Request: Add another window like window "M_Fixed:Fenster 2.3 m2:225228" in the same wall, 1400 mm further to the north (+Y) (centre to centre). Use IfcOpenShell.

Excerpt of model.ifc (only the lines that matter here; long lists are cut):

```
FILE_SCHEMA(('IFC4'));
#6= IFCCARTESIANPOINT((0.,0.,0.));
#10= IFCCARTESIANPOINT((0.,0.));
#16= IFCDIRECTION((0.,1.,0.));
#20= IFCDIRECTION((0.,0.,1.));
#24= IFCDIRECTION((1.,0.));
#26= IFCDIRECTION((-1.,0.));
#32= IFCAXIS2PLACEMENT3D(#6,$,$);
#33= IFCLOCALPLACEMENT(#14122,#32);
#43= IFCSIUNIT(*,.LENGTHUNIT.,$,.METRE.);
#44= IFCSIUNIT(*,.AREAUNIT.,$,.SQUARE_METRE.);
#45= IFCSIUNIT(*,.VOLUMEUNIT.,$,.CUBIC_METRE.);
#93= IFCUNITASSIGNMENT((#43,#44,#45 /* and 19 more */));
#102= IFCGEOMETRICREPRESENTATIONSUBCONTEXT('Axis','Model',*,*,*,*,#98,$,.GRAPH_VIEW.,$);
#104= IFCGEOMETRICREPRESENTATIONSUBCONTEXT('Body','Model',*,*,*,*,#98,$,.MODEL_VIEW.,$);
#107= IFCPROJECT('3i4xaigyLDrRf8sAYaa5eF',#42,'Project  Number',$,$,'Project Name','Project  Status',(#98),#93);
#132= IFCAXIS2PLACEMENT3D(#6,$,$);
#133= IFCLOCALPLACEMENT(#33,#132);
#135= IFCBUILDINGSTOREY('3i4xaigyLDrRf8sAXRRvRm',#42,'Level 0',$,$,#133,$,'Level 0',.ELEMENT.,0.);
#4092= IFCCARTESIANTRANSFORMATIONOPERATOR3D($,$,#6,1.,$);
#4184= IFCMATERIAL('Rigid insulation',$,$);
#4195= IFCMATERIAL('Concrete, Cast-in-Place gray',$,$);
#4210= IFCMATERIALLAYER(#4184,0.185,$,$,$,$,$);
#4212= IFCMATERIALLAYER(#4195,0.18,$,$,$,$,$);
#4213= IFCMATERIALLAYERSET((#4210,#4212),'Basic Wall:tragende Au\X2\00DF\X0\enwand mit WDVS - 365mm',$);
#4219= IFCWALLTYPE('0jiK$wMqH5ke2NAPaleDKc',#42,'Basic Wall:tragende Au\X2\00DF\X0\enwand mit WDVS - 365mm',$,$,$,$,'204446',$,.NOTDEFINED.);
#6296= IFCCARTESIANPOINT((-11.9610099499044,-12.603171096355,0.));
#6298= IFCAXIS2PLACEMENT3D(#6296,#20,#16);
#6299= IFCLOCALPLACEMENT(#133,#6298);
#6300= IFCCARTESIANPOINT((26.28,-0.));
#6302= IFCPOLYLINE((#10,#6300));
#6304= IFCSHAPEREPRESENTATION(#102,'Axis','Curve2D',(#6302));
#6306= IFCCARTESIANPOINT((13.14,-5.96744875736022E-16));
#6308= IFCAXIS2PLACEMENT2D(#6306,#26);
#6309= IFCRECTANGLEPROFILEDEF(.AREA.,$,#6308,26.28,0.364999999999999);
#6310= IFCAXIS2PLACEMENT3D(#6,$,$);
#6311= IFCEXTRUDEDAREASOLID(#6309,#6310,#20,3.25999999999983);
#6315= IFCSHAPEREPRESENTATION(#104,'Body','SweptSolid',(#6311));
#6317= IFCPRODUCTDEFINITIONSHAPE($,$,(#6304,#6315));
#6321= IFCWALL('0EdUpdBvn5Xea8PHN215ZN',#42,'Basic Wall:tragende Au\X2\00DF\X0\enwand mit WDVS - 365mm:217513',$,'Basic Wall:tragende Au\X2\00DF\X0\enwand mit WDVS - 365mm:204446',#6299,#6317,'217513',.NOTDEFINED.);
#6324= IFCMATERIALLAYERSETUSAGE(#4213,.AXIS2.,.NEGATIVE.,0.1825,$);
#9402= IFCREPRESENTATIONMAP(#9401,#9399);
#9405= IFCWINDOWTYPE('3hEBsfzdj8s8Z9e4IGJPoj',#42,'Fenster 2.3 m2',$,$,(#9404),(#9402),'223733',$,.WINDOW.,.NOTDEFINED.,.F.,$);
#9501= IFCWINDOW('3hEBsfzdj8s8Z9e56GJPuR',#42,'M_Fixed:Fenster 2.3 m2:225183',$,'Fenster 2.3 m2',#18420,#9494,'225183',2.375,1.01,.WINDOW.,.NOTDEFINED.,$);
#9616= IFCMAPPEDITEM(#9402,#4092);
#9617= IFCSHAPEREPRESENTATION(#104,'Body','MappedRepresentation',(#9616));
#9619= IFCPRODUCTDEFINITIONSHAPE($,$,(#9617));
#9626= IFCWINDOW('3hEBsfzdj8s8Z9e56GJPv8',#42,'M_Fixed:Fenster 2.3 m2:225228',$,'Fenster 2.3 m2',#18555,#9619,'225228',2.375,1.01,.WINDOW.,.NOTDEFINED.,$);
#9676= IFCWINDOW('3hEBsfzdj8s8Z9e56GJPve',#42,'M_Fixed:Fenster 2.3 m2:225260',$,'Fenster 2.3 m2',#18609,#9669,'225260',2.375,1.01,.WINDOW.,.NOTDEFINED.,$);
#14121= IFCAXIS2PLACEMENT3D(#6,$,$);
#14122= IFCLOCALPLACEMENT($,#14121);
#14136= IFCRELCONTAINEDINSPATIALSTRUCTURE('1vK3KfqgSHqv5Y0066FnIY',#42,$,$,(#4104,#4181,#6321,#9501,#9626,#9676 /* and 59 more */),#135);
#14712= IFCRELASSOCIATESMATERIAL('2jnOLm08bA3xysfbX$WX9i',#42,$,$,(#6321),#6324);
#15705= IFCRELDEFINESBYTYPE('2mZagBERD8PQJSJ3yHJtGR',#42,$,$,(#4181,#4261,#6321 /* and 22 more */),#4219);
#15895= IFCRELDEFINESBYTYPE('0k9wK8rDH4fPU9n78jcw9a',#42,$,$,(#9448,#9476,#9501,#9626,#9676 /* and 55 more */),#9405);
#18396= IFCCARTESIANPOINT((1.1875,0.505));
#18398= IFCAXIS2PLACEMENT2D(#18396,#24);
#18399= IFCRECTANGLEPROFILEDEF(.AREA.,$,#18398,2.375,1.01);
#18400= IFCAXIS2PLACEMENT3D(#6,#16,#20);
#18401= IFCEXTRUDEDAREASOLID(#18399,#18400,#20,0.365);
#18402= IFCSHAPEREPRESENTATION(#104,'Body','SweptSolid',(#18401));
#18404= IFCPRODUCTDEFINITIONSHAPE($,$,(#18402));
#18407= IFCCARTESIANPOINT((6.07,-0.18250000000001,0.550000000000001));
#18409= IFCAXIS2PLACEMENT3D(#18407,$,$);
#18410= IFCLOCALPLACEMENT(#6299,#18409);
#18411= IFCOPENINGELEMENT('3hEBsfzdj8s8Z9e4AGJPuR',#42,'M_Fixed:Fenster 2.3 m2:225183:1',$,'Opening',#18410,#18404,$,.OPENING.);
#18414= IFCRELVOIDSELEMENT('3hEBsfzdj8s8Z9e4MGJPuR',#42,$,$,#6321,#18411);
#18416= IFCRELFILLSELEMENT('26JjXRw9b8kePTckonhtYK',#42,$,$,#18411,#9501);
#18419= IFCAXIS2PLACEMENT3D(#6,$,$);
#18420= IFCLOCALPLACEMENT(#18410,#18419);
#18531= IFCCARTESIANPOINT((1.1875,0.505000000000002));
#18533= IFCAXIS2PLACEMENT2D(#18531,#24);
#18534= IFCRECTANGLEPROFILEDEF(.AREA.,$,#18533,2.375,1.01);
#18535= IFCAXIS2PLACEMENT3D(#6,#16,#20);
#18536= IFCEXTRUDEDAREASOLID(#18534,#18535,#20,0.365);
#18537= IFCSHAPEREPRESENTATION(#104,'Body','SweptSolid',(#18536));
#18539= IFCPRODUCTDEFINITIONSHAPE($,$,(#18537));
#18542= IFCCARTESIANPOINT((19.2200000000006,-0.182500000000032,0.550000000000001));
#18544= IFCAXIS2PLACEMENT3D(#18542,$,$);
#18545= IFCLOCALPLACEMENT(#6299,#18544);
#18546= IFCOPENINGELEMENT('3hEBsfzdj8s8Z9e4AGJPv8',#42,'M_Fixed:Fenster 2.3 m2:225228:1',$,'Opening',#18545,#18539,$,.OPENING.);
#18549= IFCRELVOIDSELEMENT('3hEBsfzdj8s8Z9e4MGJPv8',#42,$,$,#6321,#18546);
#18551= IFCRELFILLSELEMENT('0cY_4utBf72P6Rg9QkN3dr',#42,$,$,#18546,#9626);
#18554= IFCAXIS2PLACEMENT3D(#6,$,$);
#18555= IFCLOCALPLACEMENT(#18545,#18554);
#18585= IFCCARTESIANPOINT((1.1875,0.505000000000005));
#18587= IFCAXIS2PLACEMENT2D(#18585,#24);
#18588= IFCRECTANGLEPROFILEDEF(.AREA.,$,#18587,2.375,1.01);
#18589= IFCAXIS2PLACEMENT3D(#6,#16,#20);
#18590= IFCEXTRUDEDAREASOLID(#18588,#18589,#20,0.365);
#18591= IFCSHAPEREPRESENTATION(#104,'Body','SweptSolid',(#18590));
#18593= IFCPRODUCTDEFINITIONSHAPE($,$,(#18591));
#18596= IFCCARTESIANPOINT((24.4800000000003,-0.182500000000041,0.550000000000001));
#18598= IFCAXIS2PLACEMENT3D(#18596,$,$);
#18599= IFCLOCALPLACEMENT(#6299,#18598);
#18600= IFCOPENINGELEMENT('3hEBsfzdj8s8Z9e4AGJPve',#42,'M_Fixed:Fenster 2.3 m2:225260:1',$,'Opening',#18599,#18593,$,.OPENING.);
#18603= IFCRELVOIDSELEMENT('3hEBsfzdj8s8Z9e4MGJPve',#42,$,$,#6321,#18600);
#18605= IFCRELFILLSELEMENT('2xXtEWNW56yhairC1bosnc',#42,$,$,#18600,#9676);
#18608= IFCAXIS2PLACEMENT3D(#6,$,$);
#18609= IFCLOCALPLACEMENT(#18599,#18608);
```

```python
import ifcopenshell
import ifcopenshell.api.feature
import ifcopenshell.api.geometry
import ifcopenshell.api.root
import ifcopenshell.geom
import ifcopenshell.util.element
import ifcopenshell.util.placement
import ifcopenshell.util.shape
import ifcopenshell.util.unit

model = ifcopenshell.open("model.ifc")
unit_scale = ifcopenshell.util.unit.calculate_unit_scale(model)
settings = ifcopenshell.geom.settings()


def volume(element):
    """Net volume in cubic metres, openings subtracted."""
    shape = ifcopenshell.geom.create_shape(settings, element)
    return ifcopenshell.util.shape.get_volume(shape.geometry)


def reuse_history(source, copy):
    """copy_class also copies each property set's owner history, people and application; keep the originals."""
    for rel in copy.IsDefinedBy:
        if rel.is_a("IfcRelDefinesByProperties") and (history := rel.RelatingPropertyDefinition.OwnerHistory):
            rel.RelatingPropertyDefinition.OwnerHistory = source.OwnerHistory
            ifcopenshell.util.element.remove_deep2(model, history)


window = model.by_guid("3hEBsfzdj8s8Z9e56GJPv8")
opening = window.FillsVoids[0].RelatingOpeningElement
wall = opening.VoidsElements[0].RelatingBuildingElement
before = volume(wall)
shift = ifcopenshell.util.placement.get_local_placement(wall.ObjectPlacement)[:3, 0] * 1.4 / unit_scale

# copy_class copies the void relationship, type, container and properties, but no geometry.
new_opening = ifcopenshell.api.root.copy_class(model, product=opening)
new_opening.Representation = ifcopenshell.util.element.copy_deep(
    model, opening.Representation, exclude=["IfcGeometricRepresentationContext", "IfcRepresentationMap"]
)
new_opening.Name = "M_Fixed:Fenster 2.3 m2"
new_window = ifcopenshell.api.root.copy_class(model, product=window)
new_window.Representation = ifcopenshell.util.element.copy_deep(
    model, window.Representation, exclude=["IfcGeometricRepresentationContext", "IfcRepresentationMap"]
)
new_window.Name = "M_Fixed:Fenster 2.3 m2"
new_window.Tag = None
reuse_history(window, new_window)
ifcopenshell.api.feature.add_filling(model, opening=new_opening, element=new_window)

for old, new in ((opening, new_opening), (window, new_window)):
    matrix = ifcopenshell.util.placement.get_local_placement(old.ObjectPlacement)
    matrix[:3, 3] += shift
    ifcopenshell.api.geometry.edit_object_placement(model, product=new, matrix=matrix, is_si=False)

after = volume(wall)

print(f"wall volume {before:.3f} -> {after:.3f} m3")

model.write("model_rev.ifc")
```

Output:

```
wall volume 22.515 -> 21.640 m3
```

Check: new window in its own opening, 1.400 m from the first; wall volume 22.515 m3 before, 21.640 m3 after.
